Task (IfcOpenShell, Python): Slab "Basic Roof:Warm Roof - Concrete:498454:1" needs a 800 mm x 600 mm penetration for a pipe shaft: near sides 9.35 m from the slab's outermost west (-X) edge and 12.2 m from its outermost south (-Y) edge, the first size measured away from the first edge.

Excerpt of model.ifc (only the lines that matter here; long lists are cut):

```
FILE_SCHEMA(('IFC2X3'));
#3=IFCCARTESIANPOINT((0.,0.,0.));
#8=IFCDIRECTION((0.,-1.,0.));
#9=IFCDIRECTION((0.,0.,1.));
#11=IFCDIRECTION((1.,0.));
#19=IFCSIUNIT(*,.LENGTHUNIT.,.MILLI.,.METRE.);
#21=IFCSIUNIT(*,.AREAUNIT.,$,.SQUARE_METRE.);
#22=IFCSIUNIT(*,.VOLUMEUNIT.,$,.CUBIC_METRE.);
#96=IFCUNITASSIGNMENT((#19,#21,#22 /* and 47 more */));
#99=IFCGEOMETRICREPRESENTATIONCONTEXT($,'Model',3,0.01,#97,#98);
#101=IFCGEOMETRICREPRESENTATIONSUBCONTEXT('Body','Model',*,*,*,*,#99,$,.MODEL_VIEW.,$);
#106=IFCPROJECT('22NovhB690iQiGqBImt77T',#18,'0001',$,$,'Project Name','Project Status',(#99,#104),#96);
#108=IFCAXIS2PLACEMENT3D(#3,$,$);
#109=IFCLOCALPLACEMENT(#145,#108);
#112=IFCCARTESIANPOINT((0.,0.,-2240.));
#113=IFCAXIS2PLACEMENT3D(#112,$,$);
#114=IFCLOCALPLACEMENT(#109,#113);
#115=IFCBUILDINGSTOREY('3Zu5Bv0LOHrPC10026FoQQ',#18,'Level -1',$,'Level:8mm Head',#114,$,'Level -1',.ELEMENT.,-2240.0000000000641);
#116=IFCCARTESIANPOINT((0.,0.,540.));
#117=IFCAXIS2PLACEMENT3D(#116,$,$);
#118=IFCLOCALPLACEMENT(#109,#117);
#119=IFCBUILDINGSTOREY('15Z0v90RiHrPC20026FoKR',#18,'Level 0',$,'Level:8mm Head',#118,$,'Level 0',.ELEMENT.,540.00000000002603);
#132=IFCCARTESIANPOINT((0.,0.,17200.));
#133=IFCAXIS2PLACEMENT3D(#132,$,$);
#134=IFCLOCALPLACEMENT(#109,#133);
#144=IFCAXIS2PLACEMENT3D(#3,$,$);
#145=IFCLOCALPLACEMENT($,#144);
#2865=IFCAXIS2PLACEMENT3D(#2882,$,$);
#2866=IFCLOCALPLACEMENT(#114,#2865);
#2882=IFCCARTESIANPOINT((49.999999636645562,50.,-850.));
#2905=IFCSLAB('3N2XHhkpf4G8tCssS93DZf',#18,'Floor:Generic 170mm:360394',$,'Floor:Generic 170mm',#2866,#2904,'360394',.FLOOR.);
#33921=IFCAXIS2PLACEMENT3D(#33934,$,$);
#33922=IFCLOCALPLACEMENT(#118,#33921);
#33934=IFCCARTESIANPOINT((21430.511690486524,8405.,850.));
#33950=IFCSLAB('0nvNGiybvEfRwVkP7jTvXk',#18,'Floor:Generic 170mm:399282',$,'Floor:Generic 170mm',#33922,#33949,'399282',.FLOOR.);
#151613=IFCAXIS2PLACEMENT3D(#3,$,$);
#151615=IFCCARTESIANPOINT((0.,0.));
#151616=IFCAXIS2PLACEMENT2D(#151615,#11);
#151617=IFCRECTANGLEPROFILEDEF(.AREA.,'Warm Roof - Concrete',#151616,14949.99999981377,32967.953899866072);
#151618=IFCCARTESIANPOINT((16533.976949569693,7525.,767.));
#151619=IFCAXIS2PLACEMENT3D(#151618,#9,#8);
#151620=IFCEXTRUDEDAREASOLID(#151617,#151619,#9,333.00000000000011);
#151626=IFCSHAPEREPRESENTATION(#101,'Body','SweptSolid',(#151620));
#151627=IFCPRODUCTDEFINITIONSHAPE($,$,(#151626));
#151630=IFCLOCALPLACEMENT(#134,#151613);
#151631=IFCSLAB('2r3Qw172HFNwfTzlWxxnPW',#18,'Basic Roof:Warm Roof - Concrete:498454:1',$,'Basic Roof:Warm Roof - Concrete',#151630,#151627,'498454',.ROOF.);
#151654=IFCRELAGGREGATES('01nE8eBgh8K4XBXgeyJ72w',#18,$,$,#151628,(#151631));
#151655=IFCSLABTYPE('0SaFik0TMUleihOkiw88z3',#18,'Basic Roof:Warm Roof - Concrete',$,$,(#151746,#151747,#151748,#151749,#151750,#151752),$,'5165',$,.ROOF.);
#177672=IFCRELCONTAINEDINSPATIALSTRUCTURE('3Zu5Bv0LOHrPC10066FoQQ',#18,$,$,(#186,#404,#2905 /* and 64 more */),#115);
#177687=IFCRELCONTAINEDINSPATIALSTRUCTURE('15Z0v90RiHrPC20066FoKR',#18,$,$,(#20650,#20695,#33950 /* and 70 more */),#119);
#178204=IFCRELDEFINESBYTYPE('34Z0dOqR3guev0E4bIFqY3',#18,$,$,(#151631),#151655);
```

```python
import numpy as np
import ifcopenshell
import ifcopenshell.api.feature
import ifcopenshell.api.geometry
import ifcopenshell.api.root
import ifcopenshell.geom
import ifcopenshell.util.placement
import ifcopenshell.util.representation
import ifcopenshell.util.shape
import ifcopenshell.util.unit

model = ifcopenshell.open("model.ifc")
unit_scale = ifcopenshell.util.unit.calculate_unit_scale(model)
settings = ifcopenshell.geom.settings()


def volume(element):
    """Net volume in cubic metres, openings subtracted."""
    shape = ifcopenshell.geom.create_shape(settings, element)
    return ifcopenshell.util.shape.get_volume(shape.geometry)


slab = model.by_id(151631)
before = volume(slab)

# Extent in the slab's own axes, in metres. The edges named are its -X and -Y sides.
slab_shape = ifcopenshell.geom.create_shape(settings, slab)
vertices = ifcopenshell.util.shape.get_vertices(slab_shape.geometry)
x_min, y_min, bottom = vertices.min(axis=0)
top = vertices[:, 2].max()

opening = ifcopenshell.api.root.create_entity(model, ifc_class="IfcOpeningElement", name="Pipe shaft opening")
context = ifcopenshell.util.representation.get_context(model, "Model", "Body", "MODEL_VIEW")
width, depth = 0.8, 0.6
outline = [(0.0, 0.0), (width, 0.0), (width, depth), (0.0, depth), (0.0, 0.0)]
# Overshoot both faces by 50 mm so the cut is clean.
shape = ifcopenshell.api.geometry.add_slab_representation(
    model, context=context, depth=top - bottom + 0.1, polyline=outline
)
ifcopenshell.api.geometry.assign_representation(model, product=opening, representation=shape)

matrix = ifcopenshell.util.placement.get_local_placement(slab.ObjectPlacement)
matrix[:, 3] = matrix @ np.append(np.array([x_min + 9.35, y_min + 12.2, bottom - 0.05]) / unit_scale, 1.0)
ifcopenshell.api.geometry.edit_object_placement(model, product=opening, matrix=matrix, is_si=False)
ifcopenshell.api.feature.add_feature(model, feature=opening, element=slab)

after = volume(slab)

print(f"slab volume {before:.3f} -> {after:.3f} m3")

model.write("model_updated.ifc")
```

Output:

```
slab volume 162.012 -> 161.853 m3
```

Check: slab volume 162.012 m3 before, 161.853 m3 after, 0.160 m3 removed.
